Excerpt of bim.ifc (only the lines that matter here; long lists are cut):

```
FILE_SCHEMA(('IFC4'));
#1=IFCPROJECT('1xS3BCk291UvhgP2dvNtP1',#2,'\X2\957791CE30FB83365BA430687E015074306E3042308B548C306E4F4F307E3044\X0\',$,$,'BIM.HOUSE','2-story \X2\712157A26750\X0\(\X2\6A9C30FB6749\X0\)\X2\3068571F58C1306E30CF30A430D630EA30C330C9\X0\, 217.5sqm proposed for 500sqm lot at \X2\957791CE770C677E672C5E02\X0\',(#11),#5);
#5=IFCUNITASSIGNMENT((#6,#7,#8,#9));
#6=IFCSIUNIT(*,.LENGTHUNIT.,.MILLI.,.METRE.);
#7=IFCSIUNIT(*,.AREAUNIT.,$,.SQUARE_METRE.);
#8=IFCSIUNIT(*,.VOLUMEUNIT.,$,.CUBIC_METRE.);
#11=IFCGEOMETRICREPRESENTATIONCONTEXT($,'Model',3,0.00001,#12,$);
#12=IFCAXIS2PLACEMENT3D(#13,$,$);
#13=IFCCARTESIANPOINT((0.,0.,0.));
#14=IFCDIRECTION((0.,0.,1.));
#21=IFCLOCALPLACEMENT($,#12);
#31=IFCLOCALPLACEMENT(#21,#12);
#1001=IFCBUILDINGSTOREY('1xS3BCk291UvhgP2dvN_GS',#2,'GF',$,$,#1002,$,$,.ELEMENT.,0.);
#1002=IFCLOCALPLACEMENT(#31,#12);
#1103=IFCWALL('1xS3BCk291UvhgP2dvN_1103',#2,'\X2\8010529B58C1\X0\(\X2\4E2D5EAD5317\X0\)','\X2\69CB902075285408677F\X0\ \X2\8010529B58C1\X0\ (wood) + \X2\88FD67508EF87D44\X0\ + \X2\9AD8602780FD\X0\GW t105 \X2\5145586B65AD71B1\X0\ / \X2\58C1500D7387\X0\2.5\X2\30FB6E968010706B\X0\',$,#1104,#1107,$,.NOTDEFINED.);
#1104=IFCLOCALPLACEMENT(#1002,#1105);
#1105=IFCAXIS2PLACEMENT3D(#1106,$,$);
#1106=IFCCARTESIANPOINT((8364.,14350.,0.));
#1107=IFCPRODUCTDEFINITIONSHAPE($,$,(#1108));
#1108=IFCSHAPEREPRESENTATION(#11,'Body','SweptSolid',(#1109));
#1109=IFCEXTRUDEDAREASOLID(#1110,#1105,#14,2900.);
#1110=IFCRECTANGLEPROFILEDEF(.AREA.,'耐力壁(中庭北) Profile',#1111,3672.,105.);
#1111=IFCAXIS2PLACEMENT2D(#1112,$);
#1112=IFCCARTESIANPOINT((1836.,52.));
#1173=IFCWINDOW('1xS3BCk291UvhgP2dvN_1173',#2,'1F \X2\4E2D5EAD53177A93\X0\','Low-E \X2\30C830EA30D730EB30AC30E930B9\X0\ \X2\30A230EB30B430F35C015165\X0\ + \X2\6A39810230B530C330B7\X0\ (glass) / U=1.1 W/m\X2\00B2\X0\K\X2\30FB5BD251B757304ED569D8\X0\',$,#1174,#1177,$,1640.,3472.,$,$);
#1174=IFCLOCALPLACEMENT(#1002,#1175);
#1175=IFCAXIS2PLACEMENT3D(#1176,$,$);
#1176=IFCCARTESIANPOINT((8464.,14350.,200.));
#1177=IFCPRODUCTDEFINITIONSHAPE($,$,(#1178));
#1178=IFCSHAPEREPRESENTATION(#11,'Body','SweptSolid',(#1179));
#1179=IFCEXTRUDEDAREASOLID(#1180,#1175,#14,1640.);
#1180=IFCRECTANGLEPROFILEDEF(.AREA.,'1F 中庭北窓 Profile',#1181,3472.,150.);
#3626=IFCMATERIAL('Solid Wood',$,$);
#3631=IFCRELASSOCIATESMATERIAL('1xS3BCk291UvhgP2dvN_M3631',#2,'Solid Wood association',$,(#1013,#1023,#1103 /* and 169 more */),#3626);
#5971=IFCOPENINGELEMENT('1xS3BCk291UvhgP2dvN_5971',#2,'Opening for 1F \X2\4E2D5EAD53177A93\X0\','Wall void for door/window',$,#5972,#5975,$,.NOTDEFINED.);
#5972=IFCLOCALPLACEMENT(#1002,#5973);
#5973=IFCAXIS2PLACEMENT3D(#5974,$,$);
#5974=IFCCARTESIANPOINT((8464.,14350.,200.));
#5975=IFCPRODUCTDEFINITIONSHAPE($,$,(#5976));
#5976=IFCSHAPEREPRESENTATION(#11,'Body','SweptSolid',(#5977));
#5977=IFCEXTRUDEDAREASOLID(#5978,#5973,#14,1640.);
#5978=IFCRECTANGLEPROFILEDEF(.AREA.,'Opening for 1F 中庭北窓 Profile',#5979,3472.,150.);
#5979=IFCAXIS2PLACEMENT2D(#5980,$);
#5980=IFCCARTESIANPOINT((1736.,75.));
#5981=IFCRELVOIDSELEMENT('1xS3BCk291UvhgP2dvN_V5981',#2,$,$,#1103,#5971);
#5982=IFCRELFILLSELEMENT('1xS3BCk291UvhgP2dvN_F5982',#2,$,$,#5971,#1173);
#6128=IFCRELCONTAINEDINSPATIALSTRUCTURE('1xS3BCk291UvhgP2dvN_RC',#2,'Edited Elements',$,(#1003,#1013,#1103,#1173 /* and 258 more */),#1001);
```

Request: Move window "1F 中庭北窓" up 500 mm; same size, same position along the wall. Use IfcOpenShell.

```python
import numpy as np
import ifcopenshell
import ifcopenshell.api.geometry
import ifcopenshell.util.placement
import ifcopenshell.util.unit

model = ifcopenshell.open("bim.ifc")
unit_scale = ifcopenshell.util.unit.calculate_unit_scale(model)

window = model.by_guid("1xS3BCk291UvhgP2dvN_1173")
opening = window.FillsVoids[0].RelatingOpeningElement
dz = 0.5 / unit_scale

shift = np.array([0.0, 0.0, dz])
# The window is not placed relative to its opening, so move both.
for product in (opening, window):
    matrix = ifcopenshell.util.placement.get_local_placement(product.ObjectPlacement)
    matrix[:3, 3] += shift
    ifcopenshell.api.geometry.edit_object_placement(model, product=product, matrix=matrix, is_si=False)

print(f"moved by {dz * unit_scale:+.3f} m")

model.write("bim_updated.ifc")
```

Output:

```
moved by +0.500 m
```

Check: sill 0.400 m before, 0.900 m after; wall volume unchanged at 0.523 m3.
